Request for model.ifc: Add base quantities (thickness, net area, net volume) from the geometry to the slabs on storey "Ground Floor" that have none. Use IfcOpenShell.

First a look at what the model holds.

```python
import ifcopenshell
import ifcopenshell.util.element
import ifcopenshell.util.unit

model = ifcopenshell.open("model.ifc")
print(model.schema)
for unit_type in ("LENGTHUNIT", "AREAUNIT", "VOLUMEUNIT"):
    print(unit_type, ifcopenshell.util.unit.calculate_unit_scale(model, unit_type))
storey = next(s for s in model.by_type("IfcBuildingStorey") if s.Name == "Ground Floor")
slabs = [e for e in ifcopenshell.util.element.get_decomposition(storey) if e.is_a("IfcSlab")]
for e in sorted(slabs, key=lambda e: e.id()):
    print(e.id(), e.is_a(), e.Name, list(ifcopenshell.util.element.get_psets(e, qtos_only=True)), sep=" | ")
```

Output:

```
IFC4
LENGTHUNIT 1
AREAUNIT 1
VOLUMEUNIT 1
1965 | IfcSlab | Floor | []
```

```python
import ifcopenshell
import ifcopenshell.api.pset
import ifcopenshell.geom
import ifcopenshell.util.element
import ifcopenshell.util.shape
import ifcopenshell.util.unit

model = ifcopenshell.open("model.ifc")
unit_scale = ifcopenshell.util.unit.calculate_unit_scale(model)
area_scale = ifcopenshell.util.unit.calculate_unit_scale(model, "AREAUNIT")
volume_scale = ifcopenshell.util.unit.calculate_unit_scale(model, "VOLUMEUNIT")
settings = ifcopenshell.geom.settings()

storey = next(s for s in model.by_type("IfcBuildingStorey") if s.Name == "Ground Floor")
slabs = [e for e in ifcopenshell.util.element.get_decomposition(storey) if e.is_a("IfcSlab")]

for e in sorted(slabs, key=lambda e: e.id()):
    if ifcopenshell.util.element.get_psets(e, qtos_only=True, should_inherit=False):
        continue
    # Geometry comes back in metres, in the element's own axes.
    shape = ifcopenshell.geom.create_shape(settings, e)
    values = {
        "Width": ifcopenshell.util.shape.get_z(shape.geometry) / unit_scale,
        "NetArea": ifcopenshell.util.shape.get_footprint_area(shape.geometry) / area_scale,
        "NetVolume": ifcopenshell.util.shape.get_volume(shape.geometry) / volume_scale,
    }
    qto = ifcopenshell.api.pset.add_qto(model, product=e, name="Qto_SlabBaseQuantities")
    ifcopenshell.api.pset.edit_qto(model, qto=qto, properties=values)
    print(e.id(), {k: round(v, 3) for k, v in values.items()})

model.write("model_updated.ifc")
```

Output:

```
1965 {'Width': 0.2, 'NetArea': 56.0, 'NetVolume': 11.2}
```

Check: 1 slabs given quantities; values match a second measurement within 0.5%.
